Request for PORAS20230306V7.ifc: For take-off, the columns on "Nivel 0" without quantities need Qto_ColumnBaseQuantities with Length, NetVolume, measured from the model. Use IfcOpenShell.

First a look at what the model holds.

```python
import ifcopenshell
import ifcopenshell.util.element
import ifcopenshell.util.unit

model = ifcopenshell.open("PORAS20230306V7.ifc")
print(model.schema)
for unit_type in ("LENGTHUNIT", "AREAUNIT", "VOLUMEUNIT"):
    print(unit_type, ifcopenshell.util.unit.calculate_unit_scale(model, unit_type))
storey = next(s for s in model.by_type("IfcBuildingStorey") if s.Name == "Nivel 0")
columns = [e for e in ifcopenshell.util.element.get_decomposition(storey) if e.is_a("IfcColumn")]
for e in sorted(columns, key=lambda e: e.id()):
    print(e.id(), e.is_a(), e.Name, list(ifcopenshell.util.element.get_psets(e, qtos_only=True)), sep=" | ")
```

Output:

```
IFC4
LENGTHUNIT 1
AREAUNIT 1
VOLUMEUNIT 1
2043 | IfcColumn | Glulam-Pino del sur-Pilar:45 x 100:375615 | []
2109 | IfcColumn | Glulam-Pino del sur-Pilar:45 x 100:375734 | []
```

```python
import ifcopenshell
import ifcopenshell.api.pset
import ifcopenshell.geom
import ifcopenshell.util.element
import ifcopenshell.util.shape
import ifcopenshell.util.unit

model = ifcopenshell.open("PORAS20230306V7.ifc")
unit_scale = ifcopenshell.util.unit.calculate_unit_scale(model)
volume_scale = ifcopenshell.util.unit.calculate_unit_scale(model, "VOLUMEUNIT")
settings = ifcopenshell.geom.settings()

storey = next(s for s in model.by_type("IfcBuildingStorey") if s.Name == "Nivel 0")
columns = [e for e in ifcopenshell.util.element.get_decomposition(storey) if e.is_a("IfcColumn")]

for e in sorted(columns, key=lambda e: e.id()):
    if ifcopenshell.util.element.get_psets(e, qtos_only=True, should_inherit=False):
        continue
    # Geometry comes back in metres, in the element's own axes.
    shape = ifcopenshell.geom.create_shape(settings, e)
    values = {
        "Length": ifcopenshell.util.shape.get_z(shape.geometry) / unit_scale,
        "NetVolume": ifcopenshell.util.shape.get_volume(shape.geometry) / volume_scale,
    }
    qto = ifcopenshell.api.pset.add_qto(model, product=e, name="Qto_ColumnBaseQuantities")
    ifcopenshell.api.pset.edit_qto(model, qto=qto, properties=values)
    print(e.id(), {k: round(v, 3) for k, v in values.items()})

model.write("PORAS20230306V7_rev.ifc")
```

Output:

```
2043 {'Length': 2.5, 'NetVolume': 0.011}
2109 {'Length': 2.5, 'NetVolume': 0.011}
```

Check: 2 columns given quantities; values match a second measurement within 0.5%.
